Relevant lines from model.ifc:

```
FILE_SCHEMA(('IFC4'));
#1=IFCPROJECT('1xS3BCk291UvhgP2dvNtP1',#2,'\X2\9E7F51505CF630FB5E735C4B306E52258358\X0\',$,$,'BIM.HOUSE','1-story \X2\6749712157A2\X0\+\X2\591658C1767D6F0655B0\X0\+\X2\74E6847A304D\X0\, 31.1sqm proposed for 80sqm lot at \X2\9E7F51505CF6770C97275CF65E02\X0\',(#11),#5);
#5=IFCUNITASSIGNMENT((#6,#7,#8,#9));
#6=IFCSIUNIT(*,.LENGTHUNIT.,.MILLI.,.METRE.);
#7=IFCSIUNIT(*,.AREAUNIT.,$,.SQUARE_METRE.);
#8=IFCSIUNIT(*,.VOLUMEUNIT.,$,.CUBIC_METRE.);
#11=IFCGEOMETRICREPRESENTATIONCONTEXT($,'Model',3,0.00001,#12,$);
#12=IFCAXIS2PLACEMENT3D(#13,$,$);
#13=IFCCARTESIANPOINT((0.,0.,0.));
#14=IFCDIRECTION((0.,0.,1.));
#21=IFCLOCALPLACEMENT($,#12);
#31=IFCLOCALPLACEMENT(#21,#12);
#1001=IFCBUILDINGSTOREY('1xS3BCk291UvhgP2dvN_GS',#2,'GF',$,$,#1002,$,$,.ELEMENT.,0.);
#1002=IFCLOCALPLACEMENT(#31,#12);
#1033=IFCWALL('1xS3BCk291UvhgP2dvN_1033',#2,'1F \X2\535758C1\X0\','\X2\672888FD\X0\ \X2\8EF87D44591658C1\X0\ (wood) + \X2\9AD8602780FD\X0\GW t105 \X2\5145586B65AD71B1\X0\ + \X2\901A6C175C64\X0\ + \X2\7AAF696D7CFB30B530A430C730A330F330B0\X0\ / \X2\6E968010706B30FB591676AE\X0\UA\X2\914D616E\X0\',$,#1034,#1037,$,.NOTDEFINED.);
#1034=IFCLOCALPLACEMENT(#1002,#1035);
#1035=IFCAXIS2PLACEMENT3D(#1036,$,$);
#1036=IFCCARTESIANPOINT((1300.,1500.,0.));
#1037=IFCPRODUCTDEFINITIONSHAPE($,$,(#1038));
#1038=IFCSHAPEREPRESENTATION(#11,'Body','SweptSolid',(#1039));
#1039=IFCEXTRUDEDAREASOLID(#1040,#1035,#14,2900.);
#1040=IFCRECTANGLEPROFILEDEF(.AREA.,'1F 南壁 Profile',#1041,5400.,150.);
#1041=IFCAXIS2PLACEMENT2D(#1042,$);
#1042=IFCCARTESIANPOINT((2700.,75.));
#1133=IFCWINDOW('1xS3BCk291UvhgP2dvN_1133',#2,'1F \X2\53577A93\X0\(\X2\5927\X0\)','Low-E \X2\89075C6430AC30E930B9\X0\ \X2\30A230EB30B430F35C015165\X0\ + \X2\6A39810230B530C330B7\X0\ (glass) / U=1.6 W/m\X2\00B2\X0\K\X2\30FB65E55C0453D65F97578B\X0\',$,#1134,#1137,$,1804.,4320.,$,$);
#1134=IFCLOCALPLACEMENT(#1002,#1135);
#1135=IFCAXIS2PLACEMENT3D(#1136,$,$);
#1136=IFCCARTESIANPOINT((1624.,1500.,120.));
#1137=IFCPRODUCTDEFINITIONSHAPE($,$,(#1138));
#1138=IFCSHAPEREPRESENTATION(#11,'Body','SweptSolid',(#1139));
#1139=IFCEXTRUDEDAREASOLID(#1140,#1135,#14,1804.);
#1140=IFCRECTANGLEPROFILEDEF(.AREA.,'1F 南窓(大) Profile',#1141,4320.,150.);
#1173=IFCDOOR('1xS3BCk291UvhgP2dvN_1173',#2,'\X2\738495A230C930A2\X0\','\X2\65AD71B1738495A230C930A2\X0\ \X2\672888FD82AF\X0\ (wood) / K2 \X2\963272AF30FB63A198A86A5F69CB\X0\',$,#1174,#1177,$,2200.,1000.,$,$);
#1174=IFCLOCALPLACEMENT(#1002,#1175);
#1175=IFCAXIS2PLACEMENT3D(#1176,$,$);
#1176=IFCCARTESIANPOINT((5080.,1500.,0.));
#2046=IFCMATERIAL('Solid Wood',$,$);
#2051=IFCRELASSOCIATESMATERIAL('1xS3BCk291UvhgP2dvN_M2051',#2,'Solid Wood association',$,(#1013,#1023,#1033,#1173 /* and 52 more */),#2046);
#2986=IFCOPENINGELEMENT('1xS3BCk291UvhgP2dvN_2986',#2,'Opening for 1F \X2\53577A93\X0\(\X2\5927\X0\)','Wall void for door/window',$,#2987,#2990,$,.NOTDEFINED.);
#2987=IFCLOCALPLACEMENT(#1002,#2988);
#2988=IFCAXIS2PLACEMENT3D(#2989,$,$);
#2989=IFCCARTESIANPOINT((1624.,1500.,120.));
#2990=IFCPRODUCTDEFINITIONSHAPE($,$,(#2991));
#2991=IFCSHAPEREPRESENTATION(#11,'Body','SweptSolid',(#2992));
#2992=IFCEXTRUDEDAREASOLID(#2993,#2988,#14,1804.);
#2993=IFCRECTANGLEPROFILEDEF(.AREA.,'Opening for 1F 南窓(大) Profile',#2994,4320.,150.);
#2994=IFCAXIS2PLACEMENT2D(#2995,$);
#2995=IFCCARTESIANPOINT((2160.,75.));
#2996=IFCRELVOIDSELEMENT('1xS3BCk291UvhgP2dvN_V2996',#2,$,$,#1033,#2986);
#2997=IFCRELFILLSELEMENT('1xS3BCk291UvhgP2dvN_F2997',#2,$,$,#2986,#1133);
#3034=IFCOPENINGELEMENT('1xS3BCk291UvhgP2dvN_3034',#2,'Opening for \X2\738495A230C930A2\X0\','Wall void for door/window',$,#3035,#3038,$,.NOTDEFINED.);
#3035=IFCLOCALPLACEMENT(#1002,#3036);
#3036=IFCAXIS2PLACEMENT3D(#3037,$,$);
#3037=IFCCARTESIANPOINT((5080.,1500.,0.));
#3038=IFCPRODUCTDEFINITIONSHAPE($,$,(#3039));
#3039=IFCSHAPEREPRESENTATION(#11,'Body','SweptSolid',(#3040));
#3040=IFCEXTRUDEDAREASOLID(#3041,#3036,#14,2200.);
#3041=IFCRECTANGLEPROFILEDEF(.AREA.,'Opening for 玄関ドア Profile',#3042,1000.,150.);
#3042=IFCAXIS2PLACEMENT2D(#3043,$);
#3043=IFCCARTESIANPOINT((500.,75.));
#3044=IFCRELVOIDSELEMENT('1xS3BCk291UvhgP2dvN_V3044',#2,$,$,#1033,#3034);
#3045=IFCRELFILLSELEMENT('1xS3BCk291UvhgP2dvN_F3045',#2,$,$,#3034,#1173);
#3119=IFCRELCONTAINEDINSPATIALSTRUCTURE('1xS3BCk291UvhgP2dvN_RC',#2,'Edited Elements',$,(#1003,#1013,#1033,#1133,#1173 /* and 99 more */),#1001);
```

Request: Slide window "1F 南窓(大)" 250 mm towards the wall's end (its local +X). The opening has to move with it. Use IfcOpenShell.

```python
import ifcopenshell
import ifcopenshell.api.geometry
import ifcopenshell.util.placement
import ifcopenshell.util.unit

model = ifcopenshell.open("model.ifc")
unit_scale = ifcopenshell.util.unit.calculate_unit_scale(model)

window = model.by_id(1133)
opening = window.FillsVoids[0].RelatingOpeningElement
wall = opening.VoidsElements[0].RelatingBuildingElement

wall_matrix = ifcopenshell.util.placement.get_local_placement(wall.ObjectPlacement)
shift = wall_matrix[:3, 0] * 0.25 / unit_scale
before = ifcopenshell.util.placement.get_local_placement(window.ObjectPlacement)[:3, 3].copy()

# The window is not placed relative to its opening, so move both.
for product in (opening, window):
    matrix = ifcopenshell.util.placement.get_local_placement(product.ObjectPlacement)
    matrix[:3, 3] += shift
    ifcopenshell.api.geometry.edit_object_placement(model, product=product, matrix=matrix, is_si=False)

after = ifcopenshell.util.placement.get_local_placement(window.ObjectPlacement)[:3, 3]
print("window moved by", (after - before).round(3) + 0.0)

model.write("model_edited.ifc")
```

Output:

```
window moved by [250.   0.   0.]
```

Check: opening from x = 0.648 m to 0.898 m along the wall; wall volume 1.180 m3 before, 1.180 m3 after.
